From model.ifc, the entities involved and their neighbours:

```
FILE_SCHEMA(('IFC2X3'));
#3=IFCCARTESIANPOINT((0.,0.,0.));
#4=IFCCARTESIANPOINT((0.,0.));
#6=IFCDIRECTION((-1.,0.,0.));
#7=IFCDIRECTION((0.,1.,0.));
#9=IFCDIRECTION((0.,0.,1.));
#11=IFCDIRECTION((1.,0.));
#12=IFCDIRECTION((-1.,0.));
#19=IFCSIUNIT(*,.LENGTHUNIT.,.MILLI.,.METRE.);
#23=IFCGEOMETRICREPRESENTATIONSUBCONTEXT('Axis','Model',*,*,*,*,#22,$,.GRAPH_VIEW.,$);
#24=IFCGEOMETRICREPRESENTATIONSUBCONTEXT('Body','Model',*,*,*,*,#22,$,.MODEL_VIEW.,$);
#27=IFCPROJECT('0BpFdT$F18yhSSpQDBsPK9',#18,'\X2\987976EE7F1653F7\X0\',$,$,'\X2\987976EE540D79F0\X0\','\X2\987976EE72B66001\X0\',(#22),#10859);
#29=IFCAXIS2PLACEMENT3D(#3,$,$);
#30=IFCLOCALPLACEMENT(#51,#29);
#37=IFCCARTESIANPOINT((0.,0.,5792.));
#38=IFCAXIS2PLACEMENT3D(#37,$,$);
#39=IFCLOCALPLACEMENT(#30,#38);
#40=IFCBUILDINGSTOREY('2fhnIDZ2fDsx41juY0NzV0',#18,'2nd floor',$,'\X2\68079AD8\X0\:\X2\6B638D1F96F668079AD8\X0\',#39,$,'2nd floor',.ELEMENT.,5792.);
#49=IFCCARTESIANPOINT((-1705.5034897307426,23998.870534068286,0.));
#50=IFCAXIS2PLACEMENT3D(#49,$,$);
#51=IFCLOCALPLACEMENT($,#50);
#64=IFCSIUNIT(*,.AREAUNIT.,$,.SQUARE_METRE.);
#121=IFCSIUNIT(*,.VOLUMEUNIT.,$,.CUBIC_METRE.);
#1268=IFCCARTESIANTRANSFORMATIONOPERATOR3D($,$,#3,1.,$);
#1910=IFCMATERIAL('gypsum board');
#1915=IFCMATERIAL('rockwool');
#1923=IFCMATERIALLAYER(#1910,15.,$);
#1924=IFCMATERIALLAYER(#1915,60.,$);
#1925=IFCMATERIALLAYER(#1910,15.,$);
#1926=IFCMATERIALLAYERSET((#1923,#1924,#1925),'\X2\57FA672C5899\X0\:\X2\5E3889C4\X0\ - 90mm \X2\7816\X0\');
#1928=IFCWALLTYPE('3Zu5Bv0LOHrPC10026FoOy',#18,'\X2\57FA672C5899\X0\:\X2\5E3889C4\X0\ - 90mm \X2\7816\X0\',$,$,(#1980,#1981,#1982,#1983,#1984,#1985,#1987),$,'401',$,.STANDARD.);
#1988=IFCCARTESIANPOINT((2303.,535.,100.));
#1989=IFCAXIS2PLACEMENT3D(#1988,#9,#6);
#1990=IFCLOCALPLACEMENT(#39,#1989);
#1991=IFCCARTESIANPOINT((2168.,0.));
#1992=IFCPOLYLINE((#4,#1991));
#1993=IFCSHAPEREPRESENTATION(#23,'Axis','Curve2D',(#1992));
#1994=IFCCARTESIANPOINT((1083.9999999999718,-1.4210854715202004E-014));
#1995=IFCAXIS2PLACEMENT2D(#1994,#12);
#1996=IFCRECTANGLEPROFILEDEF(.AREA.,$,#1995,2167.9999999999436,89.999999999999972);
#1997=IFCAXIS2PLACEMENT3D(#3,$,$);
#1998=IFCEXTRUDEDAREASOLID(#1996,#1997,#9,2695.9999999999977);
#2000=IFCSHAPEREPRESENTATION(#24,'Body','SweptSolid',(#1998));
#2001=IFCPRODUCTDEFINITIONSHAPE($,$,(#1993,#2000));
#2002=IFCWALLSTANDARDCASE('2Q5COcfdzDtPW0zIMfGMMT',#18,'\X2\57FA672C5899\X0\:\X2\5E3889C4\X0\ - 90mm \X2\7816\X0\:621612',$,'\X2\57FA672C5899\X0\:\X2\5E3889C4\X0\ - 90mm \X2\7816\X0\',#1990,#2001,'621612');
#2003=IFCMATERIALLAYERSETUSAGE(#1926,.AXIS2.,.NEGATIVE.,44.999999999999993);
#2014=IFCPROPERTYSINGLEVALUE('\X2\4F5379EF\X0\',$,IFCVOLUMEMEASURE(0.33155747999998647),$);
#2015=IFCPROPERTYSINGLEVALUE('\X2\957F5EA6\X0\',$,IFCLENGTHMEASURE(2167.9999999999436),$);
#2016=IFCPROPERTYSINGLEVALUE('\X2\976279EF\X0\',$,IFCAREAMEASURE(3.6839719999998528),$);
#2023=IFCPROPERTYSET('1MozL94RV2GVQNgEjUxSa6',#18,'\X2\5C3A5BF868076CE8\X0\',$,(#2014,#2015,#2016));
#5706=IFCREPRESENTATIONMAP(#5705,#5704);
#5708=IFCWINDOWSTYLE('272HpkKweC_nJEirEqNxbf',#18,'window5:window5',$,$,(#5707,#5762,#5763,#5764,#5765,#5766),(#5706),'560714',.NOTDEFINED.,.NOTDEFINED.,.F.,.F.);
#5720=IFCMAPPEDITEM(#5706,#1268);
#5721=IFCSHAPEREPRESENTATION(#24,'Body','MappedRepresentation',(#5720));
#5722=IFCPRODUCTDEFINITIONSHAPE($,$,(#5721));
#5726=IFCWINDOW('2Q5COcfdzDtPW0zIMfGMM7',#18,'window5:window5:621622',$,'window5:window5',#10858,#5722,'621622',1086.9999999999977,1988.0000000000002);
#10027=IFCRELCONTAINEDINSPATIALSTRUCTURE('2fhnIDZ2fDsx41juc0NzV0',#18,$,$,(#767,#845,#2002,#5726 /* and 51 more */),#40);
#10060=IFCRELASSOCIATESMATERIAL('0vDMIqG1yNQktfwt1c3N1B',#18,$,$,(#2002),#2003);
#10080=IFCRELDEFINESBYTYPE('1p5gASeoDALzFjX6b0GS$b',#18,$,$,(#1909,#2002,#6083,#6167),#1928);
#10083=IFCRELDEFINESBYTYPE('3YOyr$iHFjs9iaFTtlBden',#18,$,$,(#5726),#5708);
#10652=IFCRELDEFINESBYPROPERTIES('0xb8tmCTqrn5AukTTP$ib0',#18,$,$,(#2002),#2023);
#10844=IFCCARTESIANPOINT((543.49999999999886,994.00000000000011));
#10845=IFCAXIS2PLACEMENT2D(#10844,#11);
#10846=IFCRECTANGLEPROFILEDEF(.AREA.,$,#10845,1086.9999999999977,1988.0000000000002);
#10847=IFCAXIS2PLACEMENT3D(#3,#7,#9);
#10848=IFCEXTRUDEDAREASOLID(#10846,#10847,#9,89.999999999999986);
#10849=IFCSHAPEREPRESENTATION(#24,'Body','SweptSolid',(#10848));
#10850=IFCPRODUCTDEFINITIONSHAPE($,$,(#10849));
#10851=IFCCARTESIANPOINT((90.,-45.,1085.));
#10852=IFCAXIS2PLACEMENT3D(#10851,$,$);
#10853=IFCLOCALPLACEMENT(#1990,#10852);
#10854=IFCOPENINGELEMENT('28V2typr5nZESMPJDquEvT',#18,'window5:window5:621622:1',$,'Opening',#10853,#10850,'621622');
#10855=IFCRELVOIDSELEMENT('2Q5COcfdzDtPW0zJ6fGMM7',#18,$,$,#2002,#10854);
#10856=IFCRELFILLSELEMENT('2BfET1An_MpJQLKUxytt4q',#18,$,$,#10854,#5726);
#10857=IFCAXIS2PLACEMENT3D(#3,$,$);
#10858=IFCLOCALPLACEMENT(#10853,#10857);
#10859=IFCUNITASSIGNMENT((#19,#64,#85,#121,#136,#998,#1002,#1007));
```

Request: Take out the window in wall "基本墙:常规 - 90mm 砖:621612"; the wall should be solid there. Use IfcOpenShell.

```python
import ifcopenshell
import ifcopenshell.api.feature
import ifcopenshell.api.pset
import ifcopenshell.api.root
import ifcopenshell.geom
import ifcopenshell.util.element
import ifcopenshell.util.shape
import ifcopenshell.util.unit

model = ifcopenshell.open("model.ifc")
area_scale = ifcopenshell.util.unit.calculate_unit_scale(model, "AREAUNIT")
volume_scale = ifcopenshell.util.unit.calculate_unit_scale(model, "VOLUMEUNIT")
settings = ifcopenshell.geom.settings()


def volume(element):
    """Net volume in cubic metres, openings subtracted."""
    shape = ifcopenshell.geom.create_shape(settings, element)
    return ifcopenshell.util.shape.get_volume(shape.geometry)


window = model.by_guid("2Q5COcfdzDtPW0zIMfGMM7")
opening = window.FillsVoids[0].RelatingOpeningElement
wall = opening.VoidsElements[0].RelatingBuildingElement
before = volume(wall)

ifcopenshell.api.root.remove_product(model, product=window)
ifcopenshell.api.feature.remove_feature(model, feature=opening)

after = volume(wall)
thickness = 0.09  # wall thickness in metres

# Update the wall's stored quantities.
pset = model.by_id(ifcopenshell.util.element.get_pset(wall, "尺寸标注", should_inherit=False)["id"])
ifcopenshell.api.pset.edit_pset(model, pset=pset, properties={
    "体积": model.create_entity("IfcVolumeMeasure", after / volume_scale),
    "面积": model.create_entity("IfcAreaMeasure", after / thickness / area_scale),
})

print(f"wall volume {before:.3f} -> {after:.3f} m3")

model.write("model_edited.ifc")
```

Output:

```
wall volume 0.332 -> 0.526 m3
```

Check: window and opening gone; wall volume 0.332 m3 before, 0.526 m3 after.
